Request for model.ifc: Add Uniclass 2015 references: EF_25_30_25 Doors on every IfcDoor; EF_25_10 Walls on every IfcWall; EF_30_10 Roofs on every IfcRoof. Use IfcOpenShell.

First a look at what the model holds.

```python
import ifcopenshell

model = ifcopenshell.open("model.ifc")
print(model.schema)
print("classifications:", [c.Name for c in model.by_type("IfcClassification")])
for ifc_class in ("IfcDoor", "IfcRoof", "IfcStair", "IfcWall", "IfcWindow"):
    print(ifc_class, len(model.by_type(ifc_class)))
```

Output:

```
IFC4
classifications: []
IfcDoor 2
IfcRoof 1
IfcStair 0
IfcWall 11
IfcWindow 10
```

```python
import ifcopenshell
import ifcopenshell.api.classification

model = ifcopenshell.open("model.ifc")

system = ifcopenshell.api.classification.add_classification(model, classification="Uniclass 2015")

codes = {
    "IfcDoor": ("EF_25_30_25", "Doors"),
    "IfcWall": ("EF_25_10", "Walls"),
    "IfcRoof": ("EF_30_10", "Roofs"),
}
for ifc_class, (code, name) in codes.items():
    products = model.by_type(ifc_class)
    ifcopenshell.api.classification.add_reference(
        model, products=products, classification=system, identification=code, name=name
    )
    print(code, len(products))

model.write("model-out.ifc")
```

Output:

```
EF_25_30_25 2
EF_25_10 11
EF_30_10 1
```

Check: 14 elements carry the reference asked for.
